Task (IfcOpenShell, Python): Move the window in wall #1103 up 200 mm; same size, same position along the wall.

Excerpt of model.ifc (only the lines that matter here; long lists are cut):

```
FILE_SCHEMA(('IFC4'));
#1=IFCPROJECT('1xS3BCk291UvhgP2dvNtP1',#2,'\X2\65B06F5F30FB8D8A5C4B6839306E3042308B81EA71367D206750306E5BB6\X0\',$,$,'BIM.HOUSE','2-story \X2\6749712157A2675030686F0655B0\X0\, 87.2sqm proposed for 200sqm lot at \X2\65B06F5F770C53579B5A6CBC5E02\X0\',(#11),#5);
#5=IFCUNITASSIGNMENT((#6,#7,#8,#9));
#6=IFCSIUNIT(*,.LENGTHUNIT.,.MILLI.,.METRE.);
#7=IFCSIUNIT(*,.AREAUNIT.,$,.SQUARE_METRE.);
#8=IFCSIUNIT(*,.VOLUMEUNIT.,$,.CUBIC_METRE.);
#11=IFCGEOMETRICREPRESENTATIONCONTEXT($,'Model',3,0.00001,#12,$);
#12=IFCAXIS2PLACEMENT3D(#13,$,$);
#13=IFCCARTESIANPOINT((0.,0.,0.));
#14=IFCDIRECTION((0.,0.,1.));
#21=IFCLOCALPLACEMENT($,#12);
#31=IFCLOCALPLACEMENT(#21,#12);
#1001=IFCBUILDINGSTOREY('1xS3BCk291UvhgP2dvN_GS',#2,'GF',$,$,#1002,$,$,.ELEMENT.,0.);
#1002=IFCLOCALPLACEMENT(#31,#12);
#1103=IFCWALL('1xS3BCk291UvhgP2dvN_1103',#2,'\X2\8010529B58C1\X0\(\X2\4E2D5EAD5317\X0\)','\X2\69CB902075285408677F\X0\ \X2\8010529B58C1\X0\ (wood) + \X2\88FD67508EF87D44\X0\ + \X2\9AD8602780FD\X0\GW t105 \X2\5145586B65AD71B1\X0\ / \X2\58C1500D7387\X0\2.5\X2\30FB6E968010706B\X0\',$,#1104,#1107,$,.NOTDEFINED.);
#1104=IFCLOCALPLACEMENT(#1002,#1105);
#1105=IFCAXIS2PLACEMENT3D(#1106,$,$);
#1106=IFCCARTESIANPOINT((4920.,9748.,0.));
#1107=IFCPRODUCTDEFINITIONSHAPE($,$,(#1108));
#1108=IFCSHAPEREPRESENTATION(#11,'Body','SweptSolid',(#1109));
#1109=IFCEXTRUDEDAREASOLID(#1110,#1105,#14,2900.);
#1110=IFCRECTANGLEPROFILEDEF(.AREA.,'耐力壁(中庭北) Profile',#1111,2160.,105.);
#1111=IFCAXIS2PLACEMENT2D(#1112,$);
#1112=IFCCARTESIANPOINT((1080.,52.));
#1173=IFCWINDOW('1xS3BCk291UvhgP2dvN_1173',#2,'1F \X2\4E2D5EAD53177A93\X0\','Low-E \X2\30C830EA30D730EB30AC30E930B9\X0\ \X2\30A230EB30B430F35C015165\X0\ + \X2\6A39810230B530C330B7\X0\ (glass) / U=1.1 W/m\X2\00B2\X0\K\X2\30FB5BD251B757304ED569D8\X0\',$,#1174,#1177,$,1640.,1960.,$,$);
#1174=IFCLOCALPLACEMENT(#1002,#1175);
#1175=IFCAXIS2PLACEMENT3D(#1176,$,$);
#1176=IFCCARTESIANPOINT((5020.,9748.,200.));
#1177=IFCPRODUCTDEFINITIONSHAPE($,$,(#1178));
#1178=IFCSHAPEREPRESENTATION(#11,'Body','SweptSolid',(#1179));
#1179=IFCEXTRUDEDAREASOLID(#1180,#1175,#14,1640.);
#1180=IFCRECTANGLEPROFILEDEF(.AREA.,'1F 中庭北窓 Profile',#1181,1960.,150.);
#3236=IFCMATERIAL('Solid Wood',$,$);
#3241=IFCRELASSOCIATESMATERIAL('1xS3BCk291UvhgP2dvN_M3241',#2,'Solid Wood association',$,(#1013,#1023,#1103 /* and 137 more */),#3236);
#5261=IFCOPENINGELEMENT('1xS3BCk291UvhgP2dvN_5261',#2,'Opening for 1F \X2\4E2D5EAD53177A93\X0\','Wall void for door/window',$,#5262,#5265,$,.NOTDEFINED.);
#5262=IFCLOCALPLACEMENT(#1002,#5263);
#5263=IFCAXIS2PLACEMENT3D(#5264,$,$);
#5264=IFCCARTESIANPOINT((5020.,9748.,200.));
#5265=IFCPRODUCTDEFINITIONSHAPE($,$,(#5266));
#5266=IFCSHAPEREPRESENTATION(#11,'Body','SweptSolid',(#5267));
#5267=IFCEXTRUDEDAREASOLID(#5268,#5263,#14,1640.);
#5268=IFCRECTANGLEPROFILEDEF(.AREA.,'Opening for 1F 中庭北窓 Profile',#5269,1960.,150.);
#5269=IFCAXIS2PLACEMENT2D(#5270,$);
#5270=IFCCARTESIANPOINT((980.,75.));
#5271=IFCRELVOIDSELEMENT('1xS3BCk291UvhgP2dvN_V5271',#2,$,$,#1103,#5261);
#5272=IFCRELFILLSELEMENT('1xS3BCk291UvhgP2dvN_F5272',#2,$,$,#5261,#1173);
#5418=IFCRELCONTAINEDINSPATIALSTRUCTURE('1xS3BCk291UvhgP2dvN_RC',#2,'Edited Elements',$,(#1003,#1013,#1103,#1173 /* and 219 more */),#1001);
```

```python
import numpy as np
import ifcopenshell
import ifcopenshell.api.geometry
import ifcopenshell.util.placement
import ifcopenshell.util.unit

model = ifcopenshell.open("model.ifc")
unit_scale = ifcopenshell.util.unit.calculate_unit_scale(model)

window = model.by_id(1173)
opening = window.FillsVoids[0].RelatingOpeningElement
dz = 200.0

shift = np.array([0.0, 0.0, dz])
# The window is not placed relative to its opening, so move both.
for product in (opening, window):
    matrix = ifcopenshell.util.placement.get_local_placement(product.ObjectPlacement)
    matrix[:3, 3] += shift
    ifcopenshell.api.geometry.edit_object_placement(model, product=product, matrix=matrix, is_si=False)

print(f"moved by {dz * unit_scale:+.3f} m")

model.write("model_edited.ifc")
```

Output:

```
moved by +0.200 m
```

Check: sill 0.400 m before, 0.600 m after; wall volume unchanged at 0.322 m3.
